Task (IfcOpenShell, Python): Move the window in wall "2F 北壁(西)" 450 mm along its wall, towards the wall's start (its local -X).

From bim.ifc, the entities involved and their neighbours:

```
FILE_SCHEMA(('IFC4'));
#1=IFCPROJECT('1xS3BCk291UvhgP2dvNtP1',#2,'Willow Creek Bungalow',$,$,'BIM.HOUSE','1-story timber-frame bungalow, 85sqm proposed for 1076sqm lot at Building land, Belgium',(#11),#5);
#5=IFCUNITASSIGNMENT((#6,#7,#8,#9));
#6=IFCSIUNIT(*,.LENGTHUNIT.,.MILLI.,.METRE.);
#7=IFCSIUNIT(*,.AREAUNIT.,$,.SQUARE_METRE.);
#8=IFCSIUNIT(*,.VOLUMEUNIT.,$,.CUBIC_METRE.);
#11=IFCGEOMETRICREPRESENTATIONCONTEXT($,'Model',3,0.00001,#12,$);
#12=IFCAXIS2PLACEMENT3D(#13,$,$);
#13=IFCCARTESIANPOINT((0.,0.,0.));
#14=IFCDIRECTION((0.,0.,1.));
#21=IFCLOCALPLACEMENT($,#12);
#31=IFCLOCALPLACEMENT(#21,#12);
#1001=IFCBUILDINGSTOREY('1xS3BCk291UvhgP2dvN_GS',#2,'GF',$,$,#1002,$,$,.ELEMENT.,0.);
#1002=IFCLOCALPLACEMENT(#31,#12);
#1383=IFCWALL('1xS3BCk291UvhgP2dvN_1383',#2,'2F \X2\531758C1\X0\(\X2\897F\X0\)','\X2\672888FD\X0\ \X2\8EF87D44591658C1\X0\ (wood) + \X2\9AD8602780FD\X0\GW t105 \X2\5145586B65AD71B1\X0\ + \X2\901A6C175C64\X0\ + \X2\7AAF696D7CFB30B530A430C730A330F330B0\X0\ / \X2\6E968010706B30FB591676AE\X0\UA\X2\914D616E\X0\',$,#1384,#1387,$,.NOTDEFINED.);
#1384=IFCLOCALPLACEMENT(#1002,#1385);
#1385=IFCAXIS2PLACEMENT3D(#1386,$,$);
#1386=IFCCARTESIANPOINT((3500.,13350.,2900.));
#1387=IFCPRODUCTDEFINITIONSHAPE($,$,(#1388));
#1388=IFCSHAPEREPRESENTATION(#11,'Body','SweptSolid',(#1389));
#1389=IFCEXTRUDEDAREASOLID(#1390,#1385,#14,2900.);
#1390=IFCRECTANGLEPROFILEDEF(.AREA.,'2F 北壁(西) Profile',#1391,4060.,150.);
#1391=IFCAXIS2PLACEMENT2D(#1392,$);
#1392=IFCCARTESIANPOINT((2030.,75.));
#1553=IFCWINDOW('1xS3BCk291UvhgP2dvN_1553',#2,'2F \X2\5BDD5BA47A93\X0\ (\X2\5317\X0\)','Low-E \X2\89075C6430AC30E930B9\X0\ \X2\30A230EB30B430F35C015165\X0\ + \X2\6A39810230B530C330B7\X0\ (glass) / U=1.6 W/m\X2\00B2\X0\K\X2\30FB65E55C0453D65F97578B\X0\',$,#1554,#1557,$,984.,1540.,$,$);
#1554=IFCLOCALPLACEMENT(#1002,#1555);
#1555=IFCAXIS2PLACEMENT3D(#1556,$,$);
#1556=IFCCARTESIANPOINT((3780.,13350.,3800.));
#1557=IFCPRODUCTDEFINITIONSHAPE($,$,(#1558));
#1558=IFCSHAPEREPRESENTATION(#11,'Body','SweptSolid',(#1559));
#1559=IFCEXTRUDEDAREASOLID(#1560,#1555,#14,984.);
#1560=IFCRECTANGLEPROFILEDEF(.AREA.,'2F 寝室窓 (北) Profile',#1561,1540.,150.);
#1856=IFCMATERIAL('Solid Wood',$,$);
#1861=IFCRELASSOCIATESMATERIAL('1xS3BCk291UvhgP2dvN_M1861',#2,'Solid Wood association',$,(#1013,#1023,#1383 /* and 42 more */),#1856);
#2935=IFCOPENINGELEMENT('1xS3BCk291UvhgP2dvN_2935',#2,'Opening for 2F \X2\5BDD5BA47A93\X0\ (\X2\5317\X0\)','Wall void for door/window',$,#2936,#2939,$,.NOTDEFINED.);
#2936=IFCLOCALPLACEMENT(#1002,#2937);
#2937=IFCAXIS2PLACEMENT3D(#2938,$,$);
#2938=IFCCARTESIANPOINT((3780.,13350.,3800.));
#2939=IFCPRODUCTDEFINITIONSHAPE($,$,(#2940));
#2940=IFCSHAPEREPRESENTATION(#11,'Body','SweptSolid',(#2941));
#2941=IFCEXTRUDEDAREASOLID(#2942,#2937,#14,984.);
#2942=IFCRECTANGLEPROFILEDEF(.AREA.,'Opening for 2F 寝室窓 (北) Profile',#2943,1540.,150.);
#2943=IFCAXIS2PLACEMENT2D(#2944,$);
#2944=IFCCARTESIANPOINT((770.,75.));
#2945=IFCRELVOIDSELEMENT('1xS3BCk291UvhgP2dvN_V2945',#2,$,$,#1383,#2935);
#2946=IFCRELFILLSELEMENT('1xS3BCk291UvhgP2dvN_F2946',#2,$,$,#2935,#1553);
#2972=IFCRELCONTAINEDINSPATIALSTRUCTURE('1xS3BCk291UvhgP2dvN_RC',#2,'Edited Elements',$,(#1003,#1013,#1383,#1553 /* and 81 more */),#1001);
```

```python
import ifcopenshell
import ifcopenshell.api.geometry
import ifcopenshell.util.placement
import ifcopenshell.util.unit

model = ifcopenshell.open("bim.ifc")
unit_scale = ifcopenshell.util.unit.calculate_unit_scale(model)

window = model.by_guid("1xS3BCk291UvhgP2dvN_1553")
opening = window.FillsVoids[0].RelatingOpeningElement
wall = opening.VoidsElements[0].RelatingBuildingElement

wall_matrix = ifcopenshell.util.placement.get_local_placement(wall.ObjectPlacement)
shift = wall_matrix[:3, 0] * -0.45 / unit_scale
before = ifcopenshell.util.placement.get_local_placement(window.ObjectPlacement)[:3, 3].copy()

# The window is not placed relative to its opening, so move both.
for product in (opening, window):
    matrix = ifcopenshell.util.placement.get_local_placement(product.ObjectPlacement)
    matrix[:3, 3] += shift
    ifcopenshell.api.geometry.edit_object_placement(model, product=product, matrix=matrix, is_si=False)

after = ifcopenshell.util.placement.get_local_placement(window.ObjectPlacement)[:3, 3]
print("window moved by", (after - before).round(3) + 0.0)

model.write("bim-out.ifc")
```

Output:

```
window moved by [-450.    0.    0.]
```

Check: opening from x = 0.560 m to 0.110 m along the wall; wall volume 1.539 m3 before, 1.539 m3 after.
